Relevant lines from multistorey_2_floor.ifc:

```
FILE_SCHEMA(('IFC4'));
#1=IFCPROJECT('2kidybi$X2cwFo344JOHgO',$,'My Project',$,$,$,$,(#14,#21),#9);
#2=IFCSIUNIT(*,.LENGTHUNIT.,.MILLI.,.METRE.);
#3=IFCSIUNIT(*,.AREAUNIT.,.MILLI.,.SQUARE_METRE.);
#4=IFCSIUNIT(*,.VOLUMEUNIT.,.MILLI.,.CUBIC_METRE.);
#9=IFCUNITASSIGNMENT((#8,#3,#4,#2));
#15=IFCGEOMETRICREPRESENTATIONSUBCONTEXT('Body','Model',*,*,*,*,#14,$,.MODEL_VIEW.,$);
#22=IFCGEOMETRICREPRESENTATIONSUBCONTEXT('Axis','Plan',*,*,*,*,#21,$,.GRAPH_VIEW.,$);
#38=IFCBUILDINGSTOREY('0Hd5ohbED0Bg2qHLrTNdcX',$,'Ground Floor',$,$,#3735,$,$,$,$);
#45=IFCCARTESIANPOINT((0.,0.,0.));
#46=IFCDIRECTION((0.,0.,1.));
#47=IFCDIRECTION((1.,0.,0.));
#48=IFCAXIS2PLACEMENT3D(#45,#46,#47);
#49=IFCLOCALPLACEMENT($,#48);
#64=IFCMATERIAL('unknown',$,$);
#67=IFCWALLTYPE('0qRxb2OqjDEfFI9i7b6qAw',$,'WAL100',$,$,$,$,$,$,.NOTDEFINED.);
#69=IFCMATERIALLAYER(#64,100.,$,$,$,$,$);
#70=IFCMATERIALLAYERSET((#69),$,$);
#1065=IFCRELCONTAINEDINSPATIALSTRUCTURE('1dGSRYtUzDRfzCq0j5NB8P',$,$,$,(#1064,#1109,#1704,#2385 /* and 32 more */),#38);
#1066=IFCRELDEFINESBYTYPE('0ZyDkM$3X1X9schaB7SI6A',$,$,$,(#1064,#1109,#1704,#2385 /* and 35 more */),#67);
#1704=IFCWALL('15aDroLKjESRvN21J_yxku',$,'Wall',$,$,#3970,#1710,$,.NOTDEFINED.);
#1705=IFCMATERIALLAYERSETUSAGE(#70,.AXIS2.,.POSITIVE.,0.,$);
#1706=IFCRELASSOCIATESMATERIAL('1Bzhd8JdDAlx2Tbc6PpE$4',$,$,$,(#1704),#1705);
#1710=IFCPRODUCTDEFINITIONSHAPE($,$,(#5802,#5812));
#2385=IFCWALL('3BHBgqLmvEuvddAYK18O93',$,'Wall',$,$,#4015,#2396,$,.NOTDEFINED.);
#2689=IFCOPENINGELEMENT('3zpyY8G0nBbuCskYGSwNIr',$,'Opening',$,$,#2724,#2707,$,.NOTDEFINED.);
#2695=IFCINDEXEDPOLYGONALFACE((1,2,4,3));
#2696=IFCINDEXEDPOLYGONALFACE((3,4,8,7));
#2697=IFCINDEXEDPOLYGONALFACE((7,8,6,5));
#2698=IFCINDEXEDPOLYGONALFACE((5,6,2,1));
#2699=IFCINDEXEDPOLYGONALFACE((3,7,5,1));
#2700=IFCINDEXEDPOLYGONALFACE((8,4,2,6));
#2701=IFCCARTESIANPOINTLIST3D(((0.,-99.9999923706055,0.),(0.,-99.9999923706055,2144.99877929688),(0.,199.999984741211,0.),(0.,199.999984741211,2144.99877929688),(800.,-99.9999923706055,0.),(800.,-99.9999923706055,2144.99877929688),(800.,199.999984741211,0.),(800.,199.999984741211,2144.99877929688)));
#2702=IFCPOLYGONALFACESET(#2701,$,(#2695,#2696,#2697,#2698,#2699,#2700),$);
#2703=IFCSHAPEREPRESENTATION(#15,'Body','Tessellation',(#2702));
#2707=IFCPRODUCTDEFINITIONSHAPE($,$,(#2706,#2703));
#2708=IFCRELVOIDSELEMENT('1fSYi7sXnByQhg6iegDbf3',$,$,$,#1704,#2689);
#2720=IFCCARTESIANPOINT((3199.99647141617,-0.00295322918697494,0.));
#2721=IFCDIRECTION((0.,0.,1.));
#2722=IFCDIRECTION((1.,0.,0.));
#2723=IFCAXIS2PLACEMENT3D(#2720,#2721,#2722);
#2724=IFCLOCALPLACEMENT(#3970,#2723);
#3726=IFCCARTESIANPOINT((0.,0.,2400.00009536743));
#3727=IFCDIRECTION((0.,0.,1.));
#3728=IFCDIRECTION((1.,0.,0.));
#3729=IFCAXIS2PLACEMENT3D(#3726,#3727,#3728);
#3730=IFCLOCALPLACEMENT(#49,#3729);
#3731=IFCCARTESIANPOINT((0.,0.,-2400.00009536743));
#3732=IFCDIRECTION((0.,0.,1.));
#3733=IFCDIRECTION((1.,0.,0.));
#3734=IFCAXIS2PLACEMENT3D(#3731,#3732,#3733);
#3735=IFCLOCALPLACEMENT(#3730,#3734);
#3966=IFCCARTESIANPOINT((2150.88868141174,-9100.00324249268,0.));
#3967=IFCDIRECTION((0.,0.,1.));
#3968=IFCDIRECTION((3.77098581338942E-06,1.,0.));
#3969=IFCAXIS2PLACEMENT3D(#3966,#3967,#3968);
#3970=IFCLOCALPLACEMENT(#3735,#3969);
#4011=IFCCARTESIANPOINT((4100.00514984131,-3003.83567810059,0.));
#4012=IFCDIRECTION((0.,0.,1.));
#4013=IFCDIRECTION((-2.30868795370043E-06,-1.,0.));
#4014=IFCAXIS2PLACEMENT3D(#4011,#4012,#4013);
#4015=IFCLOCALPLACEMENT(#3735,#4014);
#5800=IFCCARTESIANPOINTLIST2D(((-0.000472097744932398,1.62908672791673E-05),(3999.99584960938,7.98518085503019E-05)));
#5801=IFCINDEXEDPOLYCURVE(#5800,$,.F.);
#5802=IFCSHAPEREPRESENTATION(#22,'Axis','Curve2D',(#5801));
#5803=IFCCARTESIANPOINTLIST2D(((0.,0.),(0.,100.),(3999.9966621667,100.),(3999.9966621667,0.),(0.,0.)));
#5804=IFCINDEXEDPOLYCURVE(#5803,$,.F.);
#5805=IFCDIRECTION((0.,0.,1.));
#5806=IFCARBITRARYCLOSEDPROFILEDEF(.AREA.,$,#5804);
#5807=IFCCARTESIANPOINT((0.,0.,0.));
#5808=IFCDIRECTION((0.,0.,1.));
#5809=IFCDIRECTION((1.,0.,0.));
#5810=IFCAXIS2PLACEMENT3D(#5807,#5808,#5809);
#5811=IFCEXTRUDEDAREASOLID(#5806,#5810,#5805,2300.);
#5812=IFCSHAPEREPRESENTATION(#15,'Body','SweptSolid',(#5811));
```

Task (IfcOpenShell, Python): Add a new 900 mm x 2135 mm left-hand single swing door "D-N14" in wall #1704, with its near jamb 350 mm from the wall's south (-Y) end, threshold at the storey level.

```python
import numpy as np
import ifcopenshell
import ifcopenshell.api.feature
import ifcopenshell.api.geometry
import ifcopenshell.api.root
import ifcopenshell.api.spatial
import ifcopenshell.geom
import ifcopenshell.util.element
import ifcopenshell.util.placement
import ifcopenshell.util.representation
import ifcopenshell.util.shape
import ifcopenshell.util.unit

model = ifcopenshell.open("multistorey_2_floor.ifc")
unit_scale = ifcopenshell.util.unit.calculate_unit_scale(model)
settings = ifcopenshell.geom.settings()


def volume(element):
    """Net volume in cubic metres, openings subtracted."""
    shape = ifcopenshell.geom.create_shape(settings, element)
    return ifcopenshell.util.shape.get_volume(shape.geometry)


wall = model.by_guid("15aDroLKjESRvN21J_yxku")
storey = ifcopenshell.util.element.get_container(wall, ifc_class="IfcBuildingStorey")
context = ifcopenshell.util.representation.get_context(model, "Model", "Body", "MODEL_VIEW")
before = volume(wall)

width, height, from_end, sill = 0.9, 2.135, 0.35, 0.0  # metres

# The wall runs along its own X axis, and the end named is its -X end.
wall_shape = ifcopenshell.geom.create_shape(settings, wall)
x, y, z = ifcopenshell.util.shape.get_vertices(wall_shape.geometry).T
start = x.min() + from_end
face, thickness = float(y.min()), float(y.max() - y.min())
wall_matrix = ifcopenshell.util.placement.get_local_placement(wall.ObjectPlacement)
level = ifcopenshell.util.placement.get_local_placement(storey.ObjectPlacement)[2, 3]


def in_wall(x, y):
    """Placement at x, y metres in the wall's axes, at sill height."""
    matrix = wall_matrix.copy()
    matrix[:, 3] = wall_matrix @ np.array([x / unit_scale, y / unit_scale, 0.0, 1.0])
    matrix[2, 3] = level + sill / unit_scale
    return matrix


# Opening: a box that overshoots both wall faces by 50 mm.
opening = ifcopenshell.api.root.create_entity(model, ifc_class="IfcOpeningElement", predefined_type="OPENING")
box = ifcopenshell.api.geometry.add_wall_representation(
    model, context=context, length=width, height=height, thickness=thickness + 0.1
)
ifcopenshell.api.geometry.assign_representation(model, product=opening, representation=box)
ifcopenshell.api.geometry.edit_object_placement(model, product=opening, matrix=in_wall(start, face - 0.05), is_si=False)
ifcopenshell.api.feature.add_feature(model, feature=opening, element=wall)

door = ifcopenshell.api.root.create_entity(model, ifc_class="IfcDoor", name="D-N14", predefined_type="DOOR")
door.OverallWidth, door.OverallHeight = width / unit_scale, height / unit_scale
door.OperationType = "SINGLE_SWING_LEFT"
body = ifcopenshell.api.geometry.add_door_representation(
    model,
    context=context,
    overall_width=door.OverallWidth,
    overall_height=door.OverallHeight,
    operation_type="SINGLE_SWING_LEFT",
    lining_properties={"LiningDepth": thickness / unit_scale, "ThresholdDepth": thickness / unit_scale},
)
ifcopenshell.api.geometry.assign_representation(model, product=door, representation=body)
ifcopenshell.api.spatial.assign_container(model, products=[door], relating_structure=storey)
ifcopenshell.api.feature.add_filling(model, opening=opening, element=door)

# The lining spans the wall, so the door starts at the wall face.
ifcopenshell.api.geometry.edit_object_placement(model, product=door, matrix=in_wall(start, face), is_si=False)

after = volume(wall)

print(f"wall volume {before:.3f} -> {after:.3f} m3")

model.write("multistorey_2_floor_rev.ifc")
```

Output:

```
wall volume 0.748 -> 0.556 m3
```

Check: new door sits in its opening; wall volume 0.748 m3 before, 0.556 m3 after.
